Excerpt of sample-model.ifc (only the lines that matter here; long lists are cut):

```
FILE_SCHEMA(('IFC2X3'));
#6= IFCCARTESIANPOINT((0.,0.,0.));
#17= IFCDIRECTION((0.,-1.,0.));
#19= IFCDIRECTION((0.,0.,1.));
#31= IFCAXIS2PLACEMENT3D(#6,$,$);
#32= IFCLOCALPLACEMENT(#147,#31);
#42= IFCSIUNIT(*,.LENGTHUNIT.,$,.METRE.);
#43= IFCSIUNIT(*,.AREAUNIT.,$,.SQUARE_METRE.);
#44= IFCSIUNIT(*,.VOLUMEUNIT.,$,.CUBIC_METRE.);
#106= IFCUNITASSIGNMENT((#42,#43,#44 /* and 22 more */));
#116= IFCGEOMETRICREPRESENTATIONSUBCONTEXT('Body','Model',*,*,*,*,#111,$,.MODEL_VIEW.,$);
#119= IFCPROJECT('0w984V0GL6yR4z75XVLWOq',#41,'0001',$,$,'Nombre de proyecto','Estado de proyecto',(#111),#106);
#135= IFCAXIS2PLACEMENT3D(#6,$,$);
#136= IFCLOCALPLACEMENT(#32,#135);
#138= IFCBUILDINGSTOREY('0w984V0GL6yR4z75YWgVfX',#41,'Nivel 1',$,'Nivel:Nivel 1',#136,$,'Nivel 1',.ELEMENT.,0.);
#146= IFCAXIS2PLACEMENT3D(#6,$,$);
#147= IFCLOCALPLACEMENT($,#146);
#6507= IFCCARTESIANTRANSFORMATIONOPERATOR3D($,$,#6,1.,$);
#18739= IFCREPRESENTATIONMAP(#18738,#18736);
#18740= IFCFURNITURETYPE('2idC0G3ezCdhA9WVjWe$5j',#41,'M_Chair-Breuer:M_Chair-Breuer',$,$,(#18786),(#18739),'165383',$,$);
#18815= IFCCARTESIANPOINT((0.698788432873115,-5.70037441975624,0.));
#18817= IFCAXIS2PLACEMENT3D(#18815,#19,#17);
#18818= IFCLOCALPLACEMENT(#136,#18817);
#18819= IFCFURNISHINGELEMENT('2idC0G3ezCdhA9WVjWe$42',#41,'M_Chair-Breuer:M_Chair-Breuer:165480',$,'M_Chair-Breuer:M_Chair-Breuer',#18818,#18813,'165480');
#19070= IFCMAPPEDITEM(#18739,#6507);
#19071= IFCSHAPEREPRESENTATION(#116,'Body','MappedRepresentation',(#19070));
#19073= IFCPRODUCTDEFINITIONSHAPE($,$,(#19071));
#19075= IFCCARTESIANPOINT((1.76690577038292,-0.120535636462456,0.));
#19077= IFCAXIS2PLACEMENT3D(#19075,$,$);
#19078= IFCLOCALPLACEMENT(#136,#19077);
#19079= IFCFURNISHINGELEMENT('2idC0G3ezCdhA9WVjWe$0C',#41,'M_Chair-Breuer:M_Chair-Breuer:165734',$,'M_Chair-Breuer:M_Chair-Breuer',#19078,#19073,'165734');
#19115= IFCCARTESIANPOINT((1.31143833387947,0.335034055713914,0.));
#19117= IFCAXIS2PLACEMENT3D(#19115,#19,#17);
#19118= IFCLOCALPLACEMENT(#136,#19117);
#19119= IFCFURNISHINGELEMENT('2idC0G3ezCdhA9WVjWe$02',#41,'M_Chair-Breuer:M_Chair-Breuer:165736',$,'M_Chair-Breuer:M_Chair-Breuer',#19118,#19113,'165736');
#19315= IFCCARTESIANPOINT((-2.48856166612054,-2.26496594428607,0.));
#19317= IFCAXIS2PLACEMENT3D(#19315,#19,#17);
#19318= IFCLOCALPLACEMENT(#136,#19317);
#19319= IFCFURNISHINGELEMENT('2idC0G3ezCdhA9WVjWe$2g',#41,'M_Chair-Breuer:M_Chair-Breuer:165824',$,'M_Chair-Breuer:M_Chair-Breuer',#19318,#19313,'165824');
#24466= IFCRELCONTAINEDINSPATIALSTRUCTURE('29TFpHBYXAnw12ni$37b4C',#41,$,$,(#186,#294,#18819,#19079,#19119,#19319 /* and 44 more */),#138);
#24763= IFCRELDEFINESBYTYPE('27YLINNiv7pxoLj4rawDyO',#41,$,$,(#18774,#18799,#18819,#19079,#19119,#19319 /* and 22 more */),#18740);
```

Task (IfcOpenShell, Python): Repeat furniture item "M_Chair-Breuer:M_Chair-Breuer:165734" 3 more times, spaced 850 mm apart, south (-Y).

```python
import numpy as np
import ifcopenshell
import ifcopenshell.api.geometry
import ifcopenshell.api.root
import ifcopenshell.util.element
import ifcopenshell.util.placement
import ifcopenshell.util.unit

model = ifcopenshell.open("sample-model.ifc")
unit_scale = ifcopenshell.util.unit.calculate_unit_scale(model)


def reuse_history(source, copy):
    """copy_class also copies each property set's owner history, people and application; keep the originals."""
    for rel in copy.IsDefinedBy:
        if rel.is_a("IfcRelDefinesByProperties") and (history := rel.RelatingPropertyDefinition.OwnerHistory):
            rel.RelatingPropertyDefinition.OwnerHistory = source.OwnerHistory
            ifcopenshell.util.element.remove_deep2(model, history)


source = model.by_id(19079)
base = ifcopenshell.util.placement.get_local_placement(source.ObjectPlacement)
step = np.array([0.0, -1.0, 0.0]) * 0.85 / unit_scale

for i in range(1, 4):
    copy = ifcopenshell.api.root.copy_class(model, product=source)
    copy.Representation = ifcopenshell.util.element.copy_deep(
        model, source.Representation, exclude=["IfcGeometricRepresentationContext", "IfcRepresentationMap"]
    )
    copy.Name = "M_Chair-Breuer:M_Chair-Breuer"
    copy.Tag = None
    reuse_history(source, copy)
    matrix = base.copy()
    matrix[:3, 3] += i * step
    print("added at", matrix[:3, 3].round(3) + 0.0)
    ifcopenshell.api.geometry.edit_object_placement(model, product=copy, matrix=matrix, is_si=False)

model.write("sample-model_updated.ifc")
```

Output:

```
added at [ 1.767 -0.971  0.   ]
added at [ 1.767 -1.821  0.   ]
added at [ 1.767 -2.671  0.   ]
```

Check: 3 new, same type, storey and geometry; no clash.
